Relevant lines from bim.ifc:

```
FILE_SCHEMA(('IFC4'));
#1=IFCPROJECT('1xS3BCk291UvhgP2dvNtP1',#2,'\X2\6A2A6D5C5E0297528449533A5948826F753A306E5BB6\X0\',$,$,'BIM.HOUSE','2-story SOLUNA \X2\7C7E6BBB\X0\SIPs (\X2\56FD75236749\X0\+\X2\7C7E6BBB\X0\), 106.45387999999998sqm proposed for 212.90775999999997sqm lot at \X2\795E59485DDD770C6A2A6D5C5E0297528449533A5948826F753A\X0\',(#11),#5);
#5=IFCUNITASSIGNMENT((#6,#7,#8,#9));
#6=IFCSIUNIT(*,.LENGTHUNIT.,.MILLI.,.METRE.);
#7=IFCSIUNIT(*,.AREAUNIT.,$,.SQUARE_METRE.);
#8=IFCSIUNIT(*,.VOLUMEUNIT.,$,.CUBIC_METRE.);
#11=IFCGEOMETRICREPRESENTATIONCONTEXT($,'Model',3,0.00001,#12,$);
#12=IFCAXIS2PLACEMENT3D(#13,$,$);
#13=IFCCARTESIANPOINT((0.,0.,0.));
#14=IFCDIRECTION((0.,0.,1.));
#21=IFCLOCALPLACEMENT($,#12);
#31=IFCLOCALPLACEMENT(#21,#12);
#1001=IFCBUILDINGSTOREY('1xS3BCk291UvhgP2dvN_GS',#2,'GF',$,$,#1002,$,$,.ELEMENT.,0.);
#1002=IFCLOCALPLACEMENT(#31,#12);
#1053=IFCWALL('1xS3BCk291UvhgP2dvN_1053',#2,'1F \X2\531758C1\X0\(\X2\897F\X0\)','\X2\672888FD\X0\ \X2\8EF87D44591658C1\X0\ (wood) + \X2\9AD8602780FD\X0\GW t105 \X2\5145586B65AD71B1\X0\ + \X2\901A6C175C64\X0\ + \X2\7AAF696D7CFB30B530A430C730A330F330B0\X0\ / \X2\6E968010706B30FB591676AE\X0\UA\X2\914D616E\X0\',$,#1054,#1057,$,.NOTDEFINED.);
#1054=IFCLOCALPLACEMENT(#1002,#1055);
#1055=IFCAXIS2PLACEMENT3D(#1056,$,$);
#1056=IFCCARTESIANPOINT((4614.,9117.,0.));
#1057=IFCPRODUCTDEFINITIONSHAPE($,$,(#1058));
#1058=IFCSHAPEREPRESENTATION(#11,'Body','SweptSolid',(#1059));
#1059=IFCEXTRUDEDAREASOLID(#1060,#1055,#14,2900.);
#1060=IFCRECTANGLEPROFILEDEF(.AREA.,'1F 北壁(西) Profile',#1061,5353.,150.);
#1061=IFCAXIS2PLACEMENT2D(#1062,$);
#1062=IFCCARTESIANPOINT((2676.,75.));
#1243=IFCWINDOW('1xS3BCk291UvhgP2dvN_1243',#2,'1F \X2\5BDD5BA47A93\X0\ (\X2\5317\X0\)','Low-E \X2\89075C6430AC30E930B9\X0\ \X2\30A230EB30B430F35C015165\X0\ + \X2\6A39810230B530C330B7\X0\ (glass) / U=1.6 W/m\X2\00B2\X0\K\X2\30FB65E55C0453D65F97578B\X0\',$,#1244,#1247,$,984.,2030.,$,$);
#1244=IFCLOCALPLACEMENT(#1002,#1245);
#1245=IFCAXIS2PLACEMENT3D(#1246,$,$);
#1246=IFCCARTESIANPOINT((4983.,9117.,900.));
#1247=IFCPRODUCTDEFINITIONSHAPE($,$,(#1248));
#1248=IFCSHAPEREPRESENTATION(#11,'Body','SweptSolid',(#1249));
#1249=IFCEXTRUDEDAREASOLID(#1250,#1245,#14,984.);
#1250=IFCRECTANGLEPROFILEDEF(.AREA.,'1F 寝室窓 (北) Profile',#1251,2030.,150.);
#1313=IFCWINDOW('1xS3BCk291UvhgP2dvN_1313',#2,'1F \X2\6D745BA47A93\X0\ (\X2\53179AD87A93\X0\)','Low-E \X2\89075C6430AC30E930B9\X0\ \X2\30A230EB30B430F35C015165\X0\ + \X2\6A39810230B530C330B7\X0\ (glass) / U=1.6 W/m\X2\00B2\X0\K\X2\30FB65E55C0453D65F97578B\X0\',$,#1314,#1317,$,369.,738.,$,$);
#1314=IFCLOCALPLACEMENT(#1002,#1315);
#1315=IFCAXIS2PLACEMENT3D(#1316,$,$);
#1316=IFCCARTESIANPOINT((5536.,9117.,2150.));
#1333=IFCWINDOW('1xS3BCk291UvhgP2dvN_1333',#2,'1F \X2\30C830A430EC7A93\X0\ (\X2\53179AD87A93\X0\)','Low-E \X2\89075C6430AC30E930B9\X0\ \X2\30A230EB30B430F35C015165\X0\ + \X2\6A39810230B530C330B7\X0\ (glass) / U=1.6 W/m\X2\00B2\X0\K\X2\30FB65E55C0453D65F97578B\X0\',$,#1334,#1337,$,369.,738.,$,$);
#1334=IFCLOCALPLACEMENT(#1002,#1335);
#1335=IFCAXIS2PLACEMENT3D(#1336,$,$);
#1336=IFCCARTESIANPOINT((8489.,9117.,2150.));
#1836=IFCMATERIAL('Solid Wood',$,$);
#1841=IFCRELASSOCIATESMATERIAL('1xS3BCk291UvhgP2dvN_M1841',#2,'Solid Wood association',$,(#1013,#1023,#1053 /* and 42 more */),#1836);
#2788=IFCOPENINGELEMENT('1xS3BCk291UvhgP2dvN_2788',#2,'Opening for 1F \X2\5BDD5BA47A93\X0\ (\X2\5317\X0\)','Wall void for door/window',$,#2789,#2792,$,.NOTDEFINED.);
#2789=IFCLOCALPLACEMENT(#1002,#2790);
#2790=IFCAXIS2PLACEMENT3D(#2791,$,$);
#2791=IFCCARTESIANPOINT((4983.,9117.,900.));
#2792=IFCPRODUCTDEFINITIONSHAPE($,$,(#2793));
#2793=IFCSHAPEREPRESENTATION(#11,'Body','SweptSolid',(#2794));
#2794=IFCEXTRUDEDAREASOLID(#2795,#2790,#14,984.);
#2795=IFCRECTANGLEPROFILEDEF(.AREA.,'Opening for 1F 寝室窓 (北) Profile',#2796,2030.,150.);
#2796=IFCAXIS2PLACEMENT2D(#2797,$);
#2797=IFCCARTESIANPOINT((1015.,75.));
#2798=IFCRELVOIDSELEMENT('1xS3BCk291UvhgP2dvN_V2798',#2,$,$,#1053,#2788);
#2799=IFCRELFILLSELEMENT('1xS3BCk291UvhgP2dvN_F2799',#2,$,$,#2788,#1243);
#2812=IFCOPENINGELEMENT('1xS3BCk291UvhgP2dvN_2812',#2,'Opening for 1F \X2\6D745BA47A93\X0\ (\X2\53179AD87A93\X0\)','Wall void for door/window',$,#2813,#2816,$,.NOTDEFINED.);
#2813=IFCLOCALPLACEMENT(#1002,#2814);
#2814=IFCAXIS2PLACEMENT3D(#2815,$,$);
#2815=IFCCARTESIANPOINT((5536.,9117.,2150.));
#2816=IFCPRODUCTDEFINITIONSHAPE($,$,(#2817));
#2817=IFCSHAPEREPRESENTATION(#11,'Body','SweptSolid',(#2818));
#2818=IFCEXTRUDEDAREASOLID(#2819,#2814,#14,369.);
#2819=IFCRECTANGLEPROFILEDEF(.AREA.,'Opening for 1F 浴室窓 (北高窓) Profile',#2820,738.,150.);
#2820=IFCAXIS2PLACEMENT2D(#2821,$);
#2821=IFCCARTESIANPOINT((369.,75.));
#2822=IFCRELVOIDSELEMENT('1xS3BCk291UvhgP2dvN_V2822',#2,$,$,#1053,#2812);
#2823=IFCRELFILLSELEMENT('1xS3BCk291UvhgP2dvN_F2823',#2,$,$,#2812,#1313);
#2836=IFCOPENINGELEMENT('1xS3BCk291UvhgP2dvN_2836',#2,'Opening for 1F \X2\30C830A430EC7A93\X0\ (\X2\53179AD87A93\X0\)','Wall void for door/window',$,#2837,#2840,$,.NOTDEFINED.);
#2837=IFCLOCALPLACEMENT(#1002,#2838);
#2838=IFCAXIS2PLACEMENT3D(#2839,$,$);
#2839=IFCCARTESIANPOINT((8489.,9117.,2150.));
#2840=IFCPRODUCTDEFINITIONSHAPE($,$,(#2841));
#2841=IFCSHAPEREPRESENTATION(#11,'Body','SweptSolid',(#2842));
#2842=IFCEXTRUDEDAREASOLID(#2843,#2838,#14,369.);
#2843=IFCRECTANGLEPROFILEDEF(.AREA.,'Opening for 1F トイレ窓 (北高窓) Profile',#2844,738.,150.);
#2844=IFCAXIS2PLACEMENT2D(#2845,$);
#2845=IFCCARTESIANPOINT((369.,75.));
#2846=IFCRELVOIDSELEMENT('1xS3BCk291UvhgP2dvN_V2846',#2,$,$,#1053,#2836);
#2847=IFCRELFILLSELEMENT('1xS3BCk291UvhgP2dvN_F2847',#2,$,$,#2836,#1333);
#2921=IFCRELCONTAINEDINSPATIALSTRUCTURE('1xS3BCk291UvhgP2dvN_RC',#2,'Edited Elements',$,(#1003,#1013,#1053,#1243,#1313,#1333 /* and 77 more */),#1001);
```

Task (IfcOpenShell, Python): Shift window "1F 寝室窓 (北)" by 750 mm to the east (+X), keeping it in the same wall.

```python
import ifcopenshell
import ifcopenshell.api.geometry
import ifcopenshell.util.placement

model = ifcopenshell.open("bim.ifc")

window = model.by_guid("1xS3BCk291UvhgP2dvN_1243")
opening = window.FillsVoids[0].RelatingOpeningElement
wall = opening.VoidsElements[0].RelatingBuildingElement

wall_matrix = ifcopenshell.util.placement.get_local_placement(wall.ObjectPlacement)
shift = wall_matrix[:3, 0] * 750.0
before = ifcopenshell.util.placement.get_local_placement(window.ObjectPlacement)[:3, 3].copy()

# The window is not placed relative to its opening, so move both.
for product in (opening, window):
    matrix = ifcopenshell.util.placement.get_local_placement(product.ObjectPlacement)
    matrix[:3, 3] += shift
    ifcopenshell.api.geometry.edit_object_placement(model, product=product, matrix=matrix, is_si=False)

after = ifcopenshell.util.placement.get_local_placement(window.ObjectPlacement)[:3, 3]
print("window moved by", (after - before).round(3) + 0.0)

model.write("bim_edited.ifc")
```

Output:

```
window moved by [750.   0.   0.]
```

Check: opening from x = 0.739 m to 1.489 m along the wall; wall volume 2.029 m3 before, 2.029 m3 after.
